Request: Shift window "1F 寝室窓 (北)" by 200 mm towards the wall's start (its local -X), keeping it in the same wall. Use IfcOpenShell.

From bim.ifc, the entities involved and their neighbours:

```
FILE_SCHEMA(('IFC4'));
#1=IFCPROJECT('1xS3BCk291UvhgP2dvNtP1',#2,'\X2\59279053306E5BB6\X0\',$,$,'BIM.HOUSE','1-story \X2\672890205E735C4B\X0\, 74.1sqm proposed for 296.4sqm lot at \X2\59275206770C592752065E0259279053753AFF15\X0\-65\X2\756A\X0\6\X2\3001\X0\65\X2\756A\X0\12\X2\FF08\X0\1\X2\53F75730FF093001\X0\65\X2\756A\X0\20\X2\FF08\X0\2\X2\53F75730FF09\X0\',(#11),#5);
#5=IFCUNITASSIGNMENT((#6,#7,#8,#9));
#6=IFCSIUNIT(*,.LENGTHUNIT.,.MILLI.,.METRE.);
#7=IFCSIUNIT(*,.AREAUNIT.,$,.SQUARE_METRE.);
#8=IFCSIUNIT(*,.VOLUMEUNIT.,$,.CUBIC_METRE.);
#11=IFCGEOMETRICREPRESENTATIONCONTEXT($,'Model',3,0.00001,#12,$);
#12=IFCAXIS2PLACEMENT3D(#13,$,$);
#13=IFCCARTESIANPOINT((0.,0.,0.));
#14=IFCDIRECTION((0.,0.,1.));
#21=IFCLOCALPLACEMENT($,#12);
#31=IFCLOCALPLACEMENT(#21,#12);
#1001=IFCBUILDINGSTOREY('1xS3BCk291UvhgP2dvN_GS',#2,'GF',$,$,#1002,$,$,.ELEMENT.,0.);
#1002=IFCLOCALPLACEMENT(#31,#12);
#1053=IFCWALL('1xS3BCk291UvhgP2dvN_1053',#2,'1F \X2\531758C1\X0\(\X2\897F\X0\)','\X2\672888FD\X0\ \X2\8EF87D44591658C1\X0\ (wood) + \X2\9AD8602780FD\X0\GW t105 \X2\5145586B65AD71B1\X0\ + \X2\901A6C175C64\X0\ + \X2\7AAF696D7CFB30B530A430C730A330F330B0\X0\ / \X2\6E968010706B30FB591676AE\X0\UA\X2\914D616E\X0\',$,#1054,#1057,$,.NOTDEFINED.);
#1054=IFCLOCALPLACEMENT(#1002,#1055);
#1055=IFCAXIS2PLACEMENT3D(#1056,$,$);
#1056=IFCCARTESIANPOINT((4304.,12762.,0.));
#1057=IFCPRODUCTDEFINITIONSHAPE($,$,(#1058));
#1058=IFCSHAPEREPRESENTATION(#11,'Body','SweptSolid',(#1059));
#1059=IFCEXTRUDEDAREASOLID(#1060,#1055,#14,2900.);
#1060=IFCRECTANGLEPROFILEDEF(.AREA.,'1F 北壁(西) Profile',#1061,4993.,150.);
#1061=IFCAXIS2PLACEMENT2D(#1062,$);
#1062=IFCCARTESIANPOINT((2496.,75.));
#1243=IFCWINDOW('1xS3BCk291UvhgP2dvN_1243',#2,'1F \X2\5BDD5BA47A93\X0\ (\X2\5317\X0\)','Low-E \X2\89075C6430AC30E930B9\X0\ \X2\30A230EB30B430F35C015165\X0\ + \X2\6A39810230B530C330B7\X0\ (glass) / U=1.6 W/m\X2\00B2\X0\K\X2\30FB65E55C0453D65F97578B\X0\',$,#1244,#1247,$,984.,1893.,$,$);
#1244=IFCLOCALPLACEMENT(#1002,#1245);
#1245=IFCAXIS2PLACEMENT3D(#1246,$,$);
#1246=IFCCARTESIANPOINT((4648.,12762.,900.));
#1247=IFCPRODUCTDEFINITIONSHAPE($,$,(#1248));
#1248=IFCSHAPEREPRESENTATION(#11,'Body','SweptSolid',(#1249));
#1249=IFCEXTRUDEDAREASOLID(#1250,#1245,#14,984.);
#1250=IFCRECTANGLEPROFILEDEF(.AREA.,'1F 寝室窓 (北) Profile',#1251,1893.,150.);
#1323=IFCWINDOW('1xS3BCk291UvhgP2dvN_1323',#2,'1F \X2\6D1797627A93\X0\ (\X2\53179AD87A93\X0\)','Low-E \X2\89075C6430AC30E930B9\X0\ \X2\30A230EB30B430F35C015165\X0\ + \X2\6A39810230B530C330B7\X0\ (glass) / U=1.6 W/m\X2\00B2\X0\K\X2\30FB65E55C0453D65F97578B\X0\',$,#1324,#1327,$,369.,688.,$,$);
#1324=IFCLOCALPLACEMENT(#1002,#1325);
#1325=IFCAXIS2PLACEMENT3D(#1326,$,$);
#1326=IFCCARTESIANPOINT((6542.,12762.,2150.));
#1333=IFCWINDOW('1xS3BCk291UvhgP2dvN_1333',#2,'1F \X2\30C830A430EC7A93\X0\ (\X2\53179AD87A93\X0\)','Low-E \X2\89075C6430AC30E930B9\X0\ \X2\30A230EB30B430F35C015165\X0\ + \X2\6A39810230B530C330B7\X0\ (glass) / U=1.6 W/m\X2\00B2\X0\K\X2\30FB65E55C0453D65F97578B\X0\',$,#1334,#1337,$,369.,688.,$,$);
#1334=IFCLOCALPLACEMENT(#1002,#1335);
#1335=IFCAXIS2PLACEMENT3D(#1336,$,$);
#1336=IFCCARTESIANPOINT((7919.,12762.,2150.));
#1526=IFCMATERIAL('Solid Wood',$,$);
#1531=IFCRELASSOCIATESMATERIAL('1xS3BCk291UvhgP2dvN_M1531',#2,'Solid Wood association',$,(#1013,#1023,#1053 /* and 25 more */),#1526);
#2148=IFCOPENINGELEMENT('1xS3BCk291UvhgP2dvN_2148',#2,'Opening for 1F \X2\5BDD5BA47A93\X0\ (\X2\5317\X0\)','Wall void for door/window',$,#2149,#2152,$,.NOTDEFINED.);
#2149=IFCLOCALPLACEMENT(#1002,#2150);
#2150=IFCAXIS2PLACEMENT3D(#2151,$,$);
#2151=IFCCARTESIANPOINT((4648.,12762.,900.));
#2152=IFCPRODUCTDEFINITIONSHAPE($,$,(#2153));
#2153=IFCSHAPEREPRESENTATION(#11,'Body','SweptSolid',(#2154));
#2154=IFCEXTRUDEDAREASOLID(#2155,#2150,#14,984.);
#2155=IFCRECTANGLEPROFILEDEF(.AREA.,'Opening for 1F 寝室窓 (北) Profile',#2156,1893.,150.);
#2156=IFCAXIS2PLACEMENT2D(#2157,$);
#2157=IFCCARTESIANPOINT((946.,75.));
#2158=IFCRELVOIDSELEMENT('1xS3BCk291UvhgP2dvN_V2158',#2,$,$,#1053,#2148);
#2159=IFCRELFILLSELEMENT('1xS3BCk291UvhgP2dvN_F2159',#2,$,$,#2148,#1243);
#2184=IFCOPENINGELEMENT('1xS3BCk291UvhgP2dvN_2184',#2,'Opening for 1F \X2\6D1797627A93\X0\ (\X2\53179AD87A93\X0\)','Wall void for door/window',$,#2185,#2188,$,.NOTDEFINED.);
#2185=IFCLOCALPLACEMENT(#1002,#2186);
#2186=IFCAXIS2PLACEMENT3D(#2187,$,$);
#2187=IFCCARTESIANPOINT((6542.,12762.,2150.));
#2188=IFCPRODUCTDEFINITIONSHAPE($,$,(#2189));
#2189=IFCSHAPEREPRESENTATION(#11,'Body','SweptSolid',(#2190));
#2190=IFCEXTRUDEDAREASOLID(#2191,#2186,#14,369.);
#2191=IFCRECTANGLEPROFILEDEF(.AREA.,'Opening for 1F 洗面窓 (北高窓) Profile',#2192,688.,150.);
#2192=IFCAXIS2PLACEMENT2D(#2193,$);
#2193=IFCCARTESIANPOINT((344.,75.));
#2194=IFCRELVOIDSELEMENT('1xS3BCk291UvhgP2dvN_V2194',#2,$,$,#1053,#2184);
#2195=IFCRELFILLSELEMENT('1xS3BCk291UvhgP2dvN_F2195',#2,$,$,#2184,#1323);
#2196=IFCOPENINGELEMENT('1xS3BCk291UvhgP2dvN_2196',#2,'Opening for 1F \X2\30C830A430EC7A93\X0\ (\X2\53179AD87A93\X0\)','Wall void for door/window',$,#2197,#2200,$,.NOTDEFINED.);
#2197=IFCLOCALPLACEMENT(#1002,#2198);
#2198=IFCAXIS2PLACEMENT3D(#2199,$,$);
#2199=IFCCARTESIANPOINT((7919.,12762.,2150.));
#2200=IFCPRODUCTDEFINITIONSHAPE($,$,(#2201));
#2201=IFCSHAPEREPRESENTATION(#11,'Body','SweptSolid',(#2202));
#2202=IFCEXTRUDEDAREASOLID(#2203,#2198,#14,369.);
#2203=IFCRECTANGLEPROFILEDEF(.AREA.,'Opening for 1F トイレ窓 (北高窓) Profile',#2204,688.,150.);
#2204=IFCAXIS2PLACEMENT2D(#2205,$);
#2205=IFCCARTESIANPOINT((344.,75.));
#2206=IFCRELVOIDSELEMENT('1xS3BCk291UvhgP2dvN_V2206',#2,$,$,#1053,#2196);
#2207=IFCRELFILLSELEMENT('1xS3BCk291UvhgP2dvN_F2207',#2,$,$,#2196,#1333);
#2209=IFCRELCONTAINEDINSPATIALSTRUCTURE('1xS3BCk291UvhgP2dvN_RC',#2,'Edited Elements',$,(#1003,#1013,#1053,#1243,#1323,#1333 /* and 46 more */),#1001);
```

```python
import ifcopenshell
import ifcopenshell.api.geometry
import ifcopenshell.util.placement
import ifcopenshell.util.unit

model = ifcopenshell.open("bim.ifc")
unit_scale = ifcopenshell.util.unit.calculate_unit_scale(model)

window = model.by_id(1243)
opening = window.FillsVoids[0].RelatingOpeningElement
wall = opening.VoidsElements[0].RelatingBuildingElement

wall_matrix = ifcopenshell.util.placement.get_local_placement(wall.ObjectPlacement)
shift = wall_matrix[:3, 0] * -0.2 / unit_scale
before = ifcopenshell.util.placement.get_local_placement(window.ObjectPlacement)[:3, 3].copy()

# The window is not placed relative to its opening, so move both.
for product in (opening, window):
    matrix = ifcopenshell.util.placement.get_local_placement(product.ObjectPlacement)
    matrix[:3, 3] += shift
    ifcopenshell.api.geometry.edit_object_placement(model, product=product, matrix=matrix, is_si=False)

after = ifcopenshell.util.placement.get_local_placement(window.ObjectPlacement)[:3, 3]
print("window moved by", (after - before).round(3) + 0.0)

model.write("bim-out.ifc")
```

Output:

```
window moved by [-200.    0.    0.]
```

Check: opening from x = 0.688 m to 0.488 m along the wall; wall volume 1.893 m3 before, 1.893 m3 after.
